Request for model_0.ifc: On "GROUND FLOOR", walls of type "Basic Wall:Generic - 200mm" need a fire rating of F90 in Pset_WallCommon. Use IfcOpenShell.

First a look at what the model holds.

```python
import ifcopenshell
import ifcopenshell.util.element

model = ifcopenshell.open("model_0.ifc")
print(model.schema)
storey = next(s for s in model.by_type("IfcBuildingStorey") if s.Name == "GROUND FLOOR")
walls = [e for e in ifcopenshell.util.element.get_decomposition(storey) if e.is_a("IfcWall")]
seen = {}
for e in walls:
    element_type = ifcopenshell.util.element.get_type(e)
    key = (element_type.Name if element_type != e and element_type else None, ifcopenshell.util.element.get_pset(e, "Pset_WallCommon", "FireRating"))
    seen[key] = seen.get(key, 0) + 1
for (name, value), count in sorted(seen.items(), key=str):
    print(count, "x", name, "|", value)
```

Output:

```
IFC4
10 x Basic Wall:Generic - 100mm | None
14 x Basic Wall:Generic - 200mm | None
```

```python
import ifcopenshell
import ifcopenshell.api.pset
import ifcopenshell.util.element

model = ifcopenshell.open("model_0.ifc")

storey = next(s for s in model.by_type("IfcBuildingStorey") if s.Name == "GROUND FLOOR")
walls = [e for e in ifcopenshell.util.element.get_decomposition(storey) if e.is_a("IfcWall")]

count = 0
for e in walls:
    element_type = ifcopenshell.util.element.get_type(e)
    if element_type in (None, e) or element_type.Name != "Basic Wall:Generic - 200mm":
        continue
    # add_pset returns the element's existing set when there is one.
    pset = ifcopenshell.api.pset.add_pset(model, product=e, name="Pset_WallCommon")
    ifcopenshell.api.pset.edit_pset(model, pset=pset, properties={"FireRating": "F90"})
    count += 1

print(count, "walls updated")

model.write("model_0_v2.ifc")
```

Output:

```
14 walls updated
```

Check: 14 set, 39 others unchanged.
